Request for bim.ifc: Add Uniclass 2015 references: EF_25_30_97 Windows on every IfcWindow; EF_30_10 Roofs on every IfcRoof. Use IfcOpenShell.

First a look at what the model holds.

```python
import ifcopenshell

model = ifcopenshell.open("bim.ifc")
print(model.schema)
print("classifications:", [c.Name for c in model.by_type("IfcClassification")])
for ifc_class in ("IfcDoor", "IfcRoof", "IfcStair", "IfcWall", "IfcWindow"):
    print(ifc_class, len(model.by_type(ifc_class)))
```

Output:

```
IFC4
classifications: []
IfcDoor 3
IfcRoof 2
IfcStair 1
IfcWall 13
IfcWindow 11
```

```python
import ifcopenshell
import ifcopenshell.api.classification

model = ifcopenshell.open("bim.ifc")

system = ifcopenshell.api.classification.add_classification(model, classification="Uniclass 2015")

codes = {
    "IfcWindow": ("EF_25_30_97", "Windows"),
    "IfcRoof": ("EF_30_10", "Roofs"),
}
for ifc_class, (code, name) in codes.items():
    products = model.by_type(ifc_class)
    ifcopenshell.api.classification.add_reference(
        model, products=products, classification=system, identification=code, name=name
    )
    print(code, len(products))

model.write("bim_updated.ifc")
```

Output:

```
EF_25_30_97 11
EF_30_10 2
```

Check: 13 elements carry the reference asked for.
